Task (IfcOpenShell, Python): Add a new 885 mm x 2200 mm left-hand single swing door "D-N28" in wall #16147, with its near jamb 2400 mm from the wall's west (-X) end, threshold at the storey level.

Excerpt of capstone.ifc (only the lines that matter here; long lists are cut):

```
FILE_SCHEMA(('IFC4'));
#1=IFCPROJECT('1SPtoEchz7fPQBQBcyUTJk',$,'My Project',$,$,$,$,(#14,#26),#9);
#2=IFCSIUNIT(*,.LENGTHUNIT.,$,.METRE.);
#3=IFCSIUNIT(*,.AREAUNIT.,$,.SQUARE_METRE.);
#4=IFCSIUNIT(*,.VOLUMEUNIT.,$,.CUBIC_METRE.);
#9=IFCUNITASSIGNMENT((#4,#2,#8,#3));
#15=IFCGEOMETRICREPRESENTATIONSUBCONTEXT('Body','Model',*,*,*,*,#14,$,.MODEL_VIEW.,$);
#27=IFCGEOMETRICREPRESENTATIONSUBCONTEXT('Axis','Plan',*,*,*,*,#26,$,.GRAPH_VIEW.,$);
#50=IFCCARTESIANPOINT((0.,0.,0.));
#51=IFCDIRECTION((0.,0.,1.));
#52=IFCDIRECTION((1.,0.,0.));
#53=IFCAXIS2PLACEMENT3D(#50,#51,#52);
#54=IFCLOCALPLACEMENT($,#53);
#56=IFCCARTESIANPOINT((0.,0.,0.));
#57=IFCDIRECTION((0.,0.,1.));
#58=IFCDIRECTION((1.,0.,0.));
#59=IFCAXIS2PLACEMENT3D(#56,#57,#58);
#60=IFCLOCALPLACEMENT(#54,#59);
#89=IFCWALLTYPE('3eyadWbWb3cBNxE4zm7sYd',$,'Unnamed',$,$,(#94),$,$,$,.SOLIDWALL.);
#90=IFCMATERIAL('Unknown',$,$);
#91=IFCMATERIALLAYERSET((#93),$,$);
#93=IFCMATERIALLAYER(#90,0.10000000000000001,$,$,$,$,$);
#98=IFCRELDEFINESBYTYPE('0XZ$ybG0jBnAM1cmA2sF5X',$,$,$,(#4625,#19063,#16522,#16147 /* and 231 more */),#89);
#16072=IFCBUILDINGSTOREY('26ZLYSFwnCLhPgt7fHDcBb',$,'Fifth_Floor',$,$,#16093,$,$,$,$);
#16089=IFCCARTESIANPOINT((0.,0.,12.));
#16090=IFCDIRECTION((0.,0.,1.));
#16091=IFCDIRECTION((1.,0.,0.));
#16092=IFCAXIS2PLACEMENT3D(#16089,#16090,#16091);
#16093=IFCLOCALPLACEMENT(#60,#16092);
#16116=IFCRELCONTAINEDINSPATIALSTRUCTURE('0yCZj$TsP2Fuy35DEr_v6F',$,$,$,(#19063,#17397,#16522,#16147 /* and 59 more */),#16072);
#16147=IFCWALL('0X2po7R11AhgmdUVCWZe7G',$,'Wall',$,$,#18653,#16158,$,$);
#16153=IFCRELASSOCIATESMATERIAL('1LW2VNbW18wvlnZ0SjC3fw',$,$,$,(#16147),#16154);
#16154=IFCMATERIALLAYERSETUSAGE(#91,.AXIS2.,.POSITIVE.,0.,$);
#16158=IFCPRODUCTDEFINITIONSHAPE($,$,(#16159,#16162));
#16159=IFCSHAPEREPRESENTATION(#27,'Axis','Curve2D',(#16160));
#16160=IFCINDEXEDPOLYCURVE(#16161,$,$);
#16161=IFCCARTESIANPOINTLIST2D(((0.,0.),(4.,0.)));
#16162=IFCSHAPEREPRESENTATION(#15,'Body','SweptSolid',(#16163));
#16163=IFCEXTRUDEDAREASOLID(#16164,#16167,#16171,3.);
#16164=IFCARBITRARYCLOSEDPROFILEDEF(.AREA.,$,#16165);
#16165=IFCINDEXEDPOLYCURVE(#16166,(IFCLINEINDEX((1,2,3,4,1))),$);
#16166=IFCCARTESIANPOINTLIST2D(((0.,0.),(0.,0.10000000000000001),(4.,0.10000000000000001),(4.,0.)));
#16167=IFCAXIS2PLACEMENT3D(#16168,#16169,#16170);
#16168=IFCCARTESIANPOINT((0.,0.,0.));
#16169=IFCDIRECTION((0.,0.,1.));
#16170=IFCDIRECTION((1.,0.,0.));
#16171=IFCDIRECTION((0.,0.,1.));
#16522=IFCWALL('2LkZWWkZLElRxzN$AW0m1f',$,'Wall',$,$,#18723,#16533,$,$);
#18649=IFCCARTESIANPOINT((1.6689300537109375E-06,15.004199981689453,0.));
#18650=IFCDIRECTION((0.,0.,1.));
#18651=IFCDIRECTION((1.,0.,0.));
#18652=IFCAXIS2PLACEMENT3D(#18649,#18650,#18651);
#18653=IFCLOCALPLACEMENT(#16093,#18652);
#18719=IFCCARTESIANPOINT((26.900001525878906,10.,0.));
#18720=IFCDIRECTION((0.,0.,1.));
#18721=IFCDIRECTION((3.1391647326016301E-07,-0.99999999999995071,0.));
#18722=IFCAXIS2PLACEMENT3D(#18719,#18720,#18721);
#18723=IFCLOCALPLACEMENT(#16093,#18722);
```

```python
import numpy as np
import ifcopenshell
import ifcopenshell.api.feature
import ifcopenshell.api.geometry
import ifcopenshell.api.root
import ifcopenshell.api.spatial
import ifcopenshell.geom
import ifcopenshell.util.element
import ifcopenshell.util.placement
import ifcopenshell.util.representation
import ifcopenshell.util.shape
import ifcopenshell.util.unit

model = ifcopenshell.open("capstone.ifc")
unit_scale = ifcopenshell.util.unit.calculate_unit_scale(model)
settings = ifcopenshell.geom.settings()


def volume(element):
    """Net volume in cubic metres, openings subtracted."""
    shape = ifcopenshell.geom.create_shape(settings, element)
    return ifcopenshell.util.shape.get_volume(shape.geometry)


wall = model.by_id(16147)
storey = ifcopenshell.util.element.get_container(wall, ifc_class="IfcBuildingStorey")
context = ifcopenshell.util.representation.get_context(model, "Model", "Body", "MODEL_VIEW")
before = volume(wall)

width, height, from_end, sill = 0.885, 2.2, 2.4, 0.0  # metres

# The wall runs along its own X axis, and the end named is its -X end.
wall_shape = ifcopenshell.geom.create_shape(settings, wall)
x, y, z = ifcopenshell.util.shape.get_vertices(wall_shape.geometry).T
start = x.min() + from_end
face, thickness = float(y.min()), float(y.max() - y.min())
wall_matrix = ifcopenshell.util.placement.get_local_placement(wall.ObjectPlacement)
level = ifcopenshell.util.placement.get_local_placement(storey.ObjectPlacement)[2, 3]


def in_wall(x, y):
    """Placement at x, y metres in the wall's axes, at sill height."""
    matrix = wall_matrix.copy()
    matrix[:, 3] = wall_matrix @ np.array([x / unit_scale, y / unit_scale, 0.0, 1.0])
    matrix[2, 3] = level + sill / unit_scale
    return matrix


# Opening: a box that overshoots both wall faces by 50 mm.
opening = ifcopenshell.api.root.create_entity(model, ifc_class="IfcOpeningElement", predefined_type="OPENING")
box = ifcopenshell.api.geometry.add_wall_representation(
    model, context=context, length=width, height=height, thickness=thickness + 0.1
)
ifcopenshell.api.geometry.assign_representation(model, product=opening, representation=box)
ifcopenshell.api.geometry.edit_object_placement(model, product=opening, matrix=in_wall(start, face - 0.05), is_si=False)
ifcopenshell.api.feature.add_feature(model, feature=opening, element=wall)

door = ifcopenshell.api.root.create_entity(model, ifc_class="IfcDoor", name="D-N28", predefined_type="DOOR")
door.OverallWidth, door.OverallHeight = width / unit_scale, height / unit_scale
door.OperationType = "SINGLE_SWING_LEFT"
body = ifcopenshell.api.geometry.add_door_representation(
    model,
    context=context,
    overall_width=door.OverallWidth,
    overall_height=door.OverallHeight,
    operation_type="SINGLE_SWING_LEFT",
    lining_properties={"LiningDepth": thickness / unit_scale, "ThresholdDepth": thickness / unit_scale},
)
ifcopenshell.api.geometry.assign_representation(model, product=door, representation=body)
ifcopenshell.api.spatial.assign_container(model, products=[door], relating_structure=storey)
ifcopenshell.api.feature.add_filling(model, opening=opening, element=door)

# The lining spans the wall, so the door starts at the wall face.
ifcopenshell.api.geometry.edit_object_placement(model, product=door, matrix=in_wall(start, face), is_si=False)

after = volume(wall)

print(f"wall volume {before:.3f} -> {after:.3f} m3")

model.write("capstone_v2.ifc")
```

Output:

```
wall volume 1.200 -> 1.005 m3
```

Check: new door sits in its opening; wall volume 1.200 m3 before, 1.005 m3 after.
